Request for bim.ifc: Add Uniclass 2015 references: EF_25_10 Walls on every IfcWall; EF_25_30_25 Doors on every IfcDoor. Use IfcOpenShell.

First a look at what the model holds.

```python
import ifcopenshell

model = ifcopenshell.open("bim.ifc")
print(model.schema)
print("classifications:", [c.Name for c in model.by_type("IfcClassification")])
for ifc_class in ("IfcDoor", "IfcRoof", "IfcStair", "IfcWall", "IfcWindow"):
    print(ifc_class, len(model.by_type(ifc_class)))
```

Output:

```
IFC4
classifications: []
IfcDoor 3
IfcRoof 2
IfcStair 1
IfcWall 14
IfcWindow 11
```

```python
import ifcopenshell
import ifcopenshell.api.classification

model = ifcopenshell.open("bim.ifc")

system = ifcopenshell.api.classification.add_classification(model, classification="Uniclass 2015")

codes = {
    "IfcWall": ("EF_25_10", "Walls"),
    "IfcDoor": ("EF_25_30_25", "Doors"),
}
for ifc_class, (code, name) in codes.items():
    products = model.by_type(ifc_class)
    ifcopenshell.api.classification.add_reference(
        model, products=products, classification=system, identification=code, name=name
    )
    print(code, len(products))

model.write("bim_updated.ifc")
```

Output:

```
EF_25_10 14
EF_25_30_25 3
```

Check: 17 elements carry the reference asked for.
